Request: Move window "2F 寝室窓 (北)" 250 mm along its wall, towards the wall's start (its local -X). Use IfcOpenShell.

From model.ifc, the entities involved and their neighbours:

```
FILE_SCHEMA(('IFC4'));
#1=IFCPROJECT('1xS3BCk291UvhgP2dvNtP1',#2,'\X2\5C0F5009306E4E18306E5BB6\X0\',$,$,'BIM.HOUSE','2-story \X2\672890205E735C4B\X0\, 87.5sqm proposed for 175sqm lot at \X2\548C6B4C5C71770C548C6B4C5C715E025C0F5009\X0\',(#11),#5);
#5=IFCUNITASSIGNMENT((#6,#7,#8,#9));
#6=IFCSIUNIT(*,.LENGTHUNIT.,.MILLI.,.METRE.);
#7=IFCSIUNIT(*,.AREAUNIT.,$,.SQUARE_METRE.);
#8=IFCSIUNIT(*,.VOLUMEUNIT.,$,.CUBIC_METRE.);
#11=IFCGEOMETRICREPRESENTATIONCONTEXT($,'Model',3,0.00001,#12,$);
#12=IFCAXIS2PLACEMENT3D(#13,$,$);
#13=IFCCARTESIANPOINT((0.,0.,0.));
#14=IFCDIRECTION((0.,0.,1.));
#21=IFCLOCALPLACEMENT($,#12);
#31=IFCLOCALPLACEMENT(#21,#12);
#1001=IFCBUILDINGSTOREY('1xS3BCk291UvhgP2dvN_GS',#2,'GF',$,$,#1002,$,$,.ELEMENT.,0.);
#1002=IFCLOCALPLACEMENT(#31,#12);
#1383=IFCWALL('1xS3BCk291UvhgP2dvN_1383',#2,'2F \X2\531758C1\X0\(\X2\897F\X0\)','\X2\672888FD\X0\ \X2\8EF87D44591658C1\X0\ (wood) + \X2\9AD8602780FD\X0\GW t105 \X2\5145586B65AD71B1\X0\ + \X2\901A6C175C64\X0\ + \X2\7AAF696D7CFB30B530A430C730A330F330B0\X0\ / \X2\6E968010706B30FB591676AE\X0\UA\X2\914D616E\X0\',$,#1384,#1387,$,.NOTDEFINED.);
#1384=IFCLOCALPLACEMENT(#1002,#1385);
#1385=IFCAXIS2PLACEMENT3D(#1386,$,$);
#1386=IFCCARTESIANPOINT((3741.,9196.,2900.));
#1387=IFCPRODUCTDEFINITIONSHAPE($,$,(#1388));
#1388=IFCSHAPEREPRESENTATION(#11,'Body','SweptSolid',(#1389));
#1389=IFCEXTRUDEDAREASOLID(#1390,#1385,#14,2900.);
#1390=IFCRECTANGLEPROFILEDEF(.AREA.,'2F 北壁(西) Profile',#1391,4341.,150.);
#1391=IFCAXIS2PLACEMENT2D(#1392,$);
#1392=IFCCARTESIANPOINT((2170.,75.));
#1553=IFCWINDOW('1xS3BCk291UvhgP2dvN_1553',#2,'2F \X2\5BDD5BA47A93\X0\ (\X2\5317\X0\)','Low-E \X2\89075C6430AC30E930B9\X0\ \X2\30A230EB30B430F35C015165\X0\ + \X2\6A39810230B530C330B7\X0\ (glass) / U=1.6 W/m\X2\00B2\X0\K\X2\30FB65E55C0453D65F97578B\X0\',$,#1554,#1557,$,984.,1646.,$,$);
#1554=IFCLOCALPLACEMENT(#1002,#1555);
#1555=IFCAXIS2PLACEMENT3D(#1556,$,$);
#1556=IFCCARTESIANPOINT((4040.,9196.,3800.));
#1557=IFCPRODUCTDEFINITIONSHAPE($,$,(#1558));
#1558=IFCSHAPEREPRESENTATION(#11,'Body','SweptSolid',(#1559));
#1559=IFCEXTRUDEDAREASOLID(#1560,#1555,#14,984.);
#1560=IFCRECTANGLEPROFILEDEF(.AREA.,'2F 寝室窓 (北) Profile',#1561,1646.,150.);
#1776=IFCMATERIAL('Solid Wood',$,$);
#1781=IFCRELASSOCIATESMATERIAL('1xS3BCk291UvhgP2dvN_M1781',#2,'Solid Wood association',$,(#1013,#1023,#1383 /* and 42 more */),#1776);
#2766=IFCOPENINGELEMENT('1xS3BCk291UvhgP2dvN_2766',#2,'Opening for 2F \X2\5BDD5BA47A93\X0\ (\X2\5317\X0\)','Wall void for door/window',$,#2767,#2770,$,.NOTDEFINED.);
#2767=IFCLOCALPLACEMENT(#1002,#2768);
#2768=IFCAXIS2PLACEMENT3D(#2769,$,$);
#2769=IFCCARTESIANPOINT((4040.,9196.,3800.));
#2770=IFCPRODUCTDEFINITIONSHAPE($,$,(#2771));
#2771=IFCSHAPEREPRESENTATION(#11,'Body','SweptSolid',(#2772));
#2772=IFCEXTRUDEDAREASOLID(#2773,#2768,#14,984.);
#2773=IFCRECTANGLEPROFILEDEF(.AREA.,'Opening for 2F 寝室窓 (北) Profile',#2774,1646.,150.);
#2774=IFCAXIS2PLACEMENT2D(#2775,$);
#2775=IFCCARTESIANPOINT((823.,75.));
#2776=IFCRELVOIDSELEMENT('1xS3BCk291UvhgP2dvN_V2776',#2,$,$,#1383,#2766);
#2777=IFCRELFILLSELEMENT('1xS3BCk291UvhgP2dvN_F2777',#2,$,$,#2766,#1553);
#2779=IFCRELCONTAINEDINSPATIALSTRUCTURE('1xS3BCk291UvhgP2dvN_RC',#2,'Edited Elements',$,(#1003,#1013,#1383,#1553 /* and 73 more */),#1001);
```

```python
import ifcopenshell
import ifcopenshell.api.geometry
import ifcopenshell.util.placement

model = ifcopenshell.open("model.ifc")

window = model.by_guid("1xS3BCk291UvhgP2dvN_1553")
opening = window.FillsVoids[0].RelatingOpeningElement
wall = opening.VoidsElements[0].RelatingBuildingElement

wall_matrix = ifcopenshell.util.placement.get_local_placement(wall.ObjectPlacement)
shift = wall_matrix[:3, 0] * -250.0
before = ifcopenshell.util.placement.get_local_placement(window.ObjectPlacement)[:3, 3].copy()

# The window is not placed relative to its opening, so move both.
for product in (opening, window):
    matrix = ifcopenshell.util.placement.get_local_placement(product.ObjectPlacement)
    matrix[:3, 3] += shift
    ifcopenshell.api.geometry.edit_object_placement(model, product=product, matrix=matrix, is_si=False)

after = ifcopenshell.util.placement.get_local_placement(window.ObjectPlacement)[:3, 3]
print("window moved by", (after - before).round(3) + 0.0)

model.write("model-out.ifc")
```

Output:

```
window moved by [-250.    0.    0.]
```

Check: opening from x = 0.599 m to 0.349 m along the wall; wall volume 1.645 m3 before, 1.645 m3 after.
